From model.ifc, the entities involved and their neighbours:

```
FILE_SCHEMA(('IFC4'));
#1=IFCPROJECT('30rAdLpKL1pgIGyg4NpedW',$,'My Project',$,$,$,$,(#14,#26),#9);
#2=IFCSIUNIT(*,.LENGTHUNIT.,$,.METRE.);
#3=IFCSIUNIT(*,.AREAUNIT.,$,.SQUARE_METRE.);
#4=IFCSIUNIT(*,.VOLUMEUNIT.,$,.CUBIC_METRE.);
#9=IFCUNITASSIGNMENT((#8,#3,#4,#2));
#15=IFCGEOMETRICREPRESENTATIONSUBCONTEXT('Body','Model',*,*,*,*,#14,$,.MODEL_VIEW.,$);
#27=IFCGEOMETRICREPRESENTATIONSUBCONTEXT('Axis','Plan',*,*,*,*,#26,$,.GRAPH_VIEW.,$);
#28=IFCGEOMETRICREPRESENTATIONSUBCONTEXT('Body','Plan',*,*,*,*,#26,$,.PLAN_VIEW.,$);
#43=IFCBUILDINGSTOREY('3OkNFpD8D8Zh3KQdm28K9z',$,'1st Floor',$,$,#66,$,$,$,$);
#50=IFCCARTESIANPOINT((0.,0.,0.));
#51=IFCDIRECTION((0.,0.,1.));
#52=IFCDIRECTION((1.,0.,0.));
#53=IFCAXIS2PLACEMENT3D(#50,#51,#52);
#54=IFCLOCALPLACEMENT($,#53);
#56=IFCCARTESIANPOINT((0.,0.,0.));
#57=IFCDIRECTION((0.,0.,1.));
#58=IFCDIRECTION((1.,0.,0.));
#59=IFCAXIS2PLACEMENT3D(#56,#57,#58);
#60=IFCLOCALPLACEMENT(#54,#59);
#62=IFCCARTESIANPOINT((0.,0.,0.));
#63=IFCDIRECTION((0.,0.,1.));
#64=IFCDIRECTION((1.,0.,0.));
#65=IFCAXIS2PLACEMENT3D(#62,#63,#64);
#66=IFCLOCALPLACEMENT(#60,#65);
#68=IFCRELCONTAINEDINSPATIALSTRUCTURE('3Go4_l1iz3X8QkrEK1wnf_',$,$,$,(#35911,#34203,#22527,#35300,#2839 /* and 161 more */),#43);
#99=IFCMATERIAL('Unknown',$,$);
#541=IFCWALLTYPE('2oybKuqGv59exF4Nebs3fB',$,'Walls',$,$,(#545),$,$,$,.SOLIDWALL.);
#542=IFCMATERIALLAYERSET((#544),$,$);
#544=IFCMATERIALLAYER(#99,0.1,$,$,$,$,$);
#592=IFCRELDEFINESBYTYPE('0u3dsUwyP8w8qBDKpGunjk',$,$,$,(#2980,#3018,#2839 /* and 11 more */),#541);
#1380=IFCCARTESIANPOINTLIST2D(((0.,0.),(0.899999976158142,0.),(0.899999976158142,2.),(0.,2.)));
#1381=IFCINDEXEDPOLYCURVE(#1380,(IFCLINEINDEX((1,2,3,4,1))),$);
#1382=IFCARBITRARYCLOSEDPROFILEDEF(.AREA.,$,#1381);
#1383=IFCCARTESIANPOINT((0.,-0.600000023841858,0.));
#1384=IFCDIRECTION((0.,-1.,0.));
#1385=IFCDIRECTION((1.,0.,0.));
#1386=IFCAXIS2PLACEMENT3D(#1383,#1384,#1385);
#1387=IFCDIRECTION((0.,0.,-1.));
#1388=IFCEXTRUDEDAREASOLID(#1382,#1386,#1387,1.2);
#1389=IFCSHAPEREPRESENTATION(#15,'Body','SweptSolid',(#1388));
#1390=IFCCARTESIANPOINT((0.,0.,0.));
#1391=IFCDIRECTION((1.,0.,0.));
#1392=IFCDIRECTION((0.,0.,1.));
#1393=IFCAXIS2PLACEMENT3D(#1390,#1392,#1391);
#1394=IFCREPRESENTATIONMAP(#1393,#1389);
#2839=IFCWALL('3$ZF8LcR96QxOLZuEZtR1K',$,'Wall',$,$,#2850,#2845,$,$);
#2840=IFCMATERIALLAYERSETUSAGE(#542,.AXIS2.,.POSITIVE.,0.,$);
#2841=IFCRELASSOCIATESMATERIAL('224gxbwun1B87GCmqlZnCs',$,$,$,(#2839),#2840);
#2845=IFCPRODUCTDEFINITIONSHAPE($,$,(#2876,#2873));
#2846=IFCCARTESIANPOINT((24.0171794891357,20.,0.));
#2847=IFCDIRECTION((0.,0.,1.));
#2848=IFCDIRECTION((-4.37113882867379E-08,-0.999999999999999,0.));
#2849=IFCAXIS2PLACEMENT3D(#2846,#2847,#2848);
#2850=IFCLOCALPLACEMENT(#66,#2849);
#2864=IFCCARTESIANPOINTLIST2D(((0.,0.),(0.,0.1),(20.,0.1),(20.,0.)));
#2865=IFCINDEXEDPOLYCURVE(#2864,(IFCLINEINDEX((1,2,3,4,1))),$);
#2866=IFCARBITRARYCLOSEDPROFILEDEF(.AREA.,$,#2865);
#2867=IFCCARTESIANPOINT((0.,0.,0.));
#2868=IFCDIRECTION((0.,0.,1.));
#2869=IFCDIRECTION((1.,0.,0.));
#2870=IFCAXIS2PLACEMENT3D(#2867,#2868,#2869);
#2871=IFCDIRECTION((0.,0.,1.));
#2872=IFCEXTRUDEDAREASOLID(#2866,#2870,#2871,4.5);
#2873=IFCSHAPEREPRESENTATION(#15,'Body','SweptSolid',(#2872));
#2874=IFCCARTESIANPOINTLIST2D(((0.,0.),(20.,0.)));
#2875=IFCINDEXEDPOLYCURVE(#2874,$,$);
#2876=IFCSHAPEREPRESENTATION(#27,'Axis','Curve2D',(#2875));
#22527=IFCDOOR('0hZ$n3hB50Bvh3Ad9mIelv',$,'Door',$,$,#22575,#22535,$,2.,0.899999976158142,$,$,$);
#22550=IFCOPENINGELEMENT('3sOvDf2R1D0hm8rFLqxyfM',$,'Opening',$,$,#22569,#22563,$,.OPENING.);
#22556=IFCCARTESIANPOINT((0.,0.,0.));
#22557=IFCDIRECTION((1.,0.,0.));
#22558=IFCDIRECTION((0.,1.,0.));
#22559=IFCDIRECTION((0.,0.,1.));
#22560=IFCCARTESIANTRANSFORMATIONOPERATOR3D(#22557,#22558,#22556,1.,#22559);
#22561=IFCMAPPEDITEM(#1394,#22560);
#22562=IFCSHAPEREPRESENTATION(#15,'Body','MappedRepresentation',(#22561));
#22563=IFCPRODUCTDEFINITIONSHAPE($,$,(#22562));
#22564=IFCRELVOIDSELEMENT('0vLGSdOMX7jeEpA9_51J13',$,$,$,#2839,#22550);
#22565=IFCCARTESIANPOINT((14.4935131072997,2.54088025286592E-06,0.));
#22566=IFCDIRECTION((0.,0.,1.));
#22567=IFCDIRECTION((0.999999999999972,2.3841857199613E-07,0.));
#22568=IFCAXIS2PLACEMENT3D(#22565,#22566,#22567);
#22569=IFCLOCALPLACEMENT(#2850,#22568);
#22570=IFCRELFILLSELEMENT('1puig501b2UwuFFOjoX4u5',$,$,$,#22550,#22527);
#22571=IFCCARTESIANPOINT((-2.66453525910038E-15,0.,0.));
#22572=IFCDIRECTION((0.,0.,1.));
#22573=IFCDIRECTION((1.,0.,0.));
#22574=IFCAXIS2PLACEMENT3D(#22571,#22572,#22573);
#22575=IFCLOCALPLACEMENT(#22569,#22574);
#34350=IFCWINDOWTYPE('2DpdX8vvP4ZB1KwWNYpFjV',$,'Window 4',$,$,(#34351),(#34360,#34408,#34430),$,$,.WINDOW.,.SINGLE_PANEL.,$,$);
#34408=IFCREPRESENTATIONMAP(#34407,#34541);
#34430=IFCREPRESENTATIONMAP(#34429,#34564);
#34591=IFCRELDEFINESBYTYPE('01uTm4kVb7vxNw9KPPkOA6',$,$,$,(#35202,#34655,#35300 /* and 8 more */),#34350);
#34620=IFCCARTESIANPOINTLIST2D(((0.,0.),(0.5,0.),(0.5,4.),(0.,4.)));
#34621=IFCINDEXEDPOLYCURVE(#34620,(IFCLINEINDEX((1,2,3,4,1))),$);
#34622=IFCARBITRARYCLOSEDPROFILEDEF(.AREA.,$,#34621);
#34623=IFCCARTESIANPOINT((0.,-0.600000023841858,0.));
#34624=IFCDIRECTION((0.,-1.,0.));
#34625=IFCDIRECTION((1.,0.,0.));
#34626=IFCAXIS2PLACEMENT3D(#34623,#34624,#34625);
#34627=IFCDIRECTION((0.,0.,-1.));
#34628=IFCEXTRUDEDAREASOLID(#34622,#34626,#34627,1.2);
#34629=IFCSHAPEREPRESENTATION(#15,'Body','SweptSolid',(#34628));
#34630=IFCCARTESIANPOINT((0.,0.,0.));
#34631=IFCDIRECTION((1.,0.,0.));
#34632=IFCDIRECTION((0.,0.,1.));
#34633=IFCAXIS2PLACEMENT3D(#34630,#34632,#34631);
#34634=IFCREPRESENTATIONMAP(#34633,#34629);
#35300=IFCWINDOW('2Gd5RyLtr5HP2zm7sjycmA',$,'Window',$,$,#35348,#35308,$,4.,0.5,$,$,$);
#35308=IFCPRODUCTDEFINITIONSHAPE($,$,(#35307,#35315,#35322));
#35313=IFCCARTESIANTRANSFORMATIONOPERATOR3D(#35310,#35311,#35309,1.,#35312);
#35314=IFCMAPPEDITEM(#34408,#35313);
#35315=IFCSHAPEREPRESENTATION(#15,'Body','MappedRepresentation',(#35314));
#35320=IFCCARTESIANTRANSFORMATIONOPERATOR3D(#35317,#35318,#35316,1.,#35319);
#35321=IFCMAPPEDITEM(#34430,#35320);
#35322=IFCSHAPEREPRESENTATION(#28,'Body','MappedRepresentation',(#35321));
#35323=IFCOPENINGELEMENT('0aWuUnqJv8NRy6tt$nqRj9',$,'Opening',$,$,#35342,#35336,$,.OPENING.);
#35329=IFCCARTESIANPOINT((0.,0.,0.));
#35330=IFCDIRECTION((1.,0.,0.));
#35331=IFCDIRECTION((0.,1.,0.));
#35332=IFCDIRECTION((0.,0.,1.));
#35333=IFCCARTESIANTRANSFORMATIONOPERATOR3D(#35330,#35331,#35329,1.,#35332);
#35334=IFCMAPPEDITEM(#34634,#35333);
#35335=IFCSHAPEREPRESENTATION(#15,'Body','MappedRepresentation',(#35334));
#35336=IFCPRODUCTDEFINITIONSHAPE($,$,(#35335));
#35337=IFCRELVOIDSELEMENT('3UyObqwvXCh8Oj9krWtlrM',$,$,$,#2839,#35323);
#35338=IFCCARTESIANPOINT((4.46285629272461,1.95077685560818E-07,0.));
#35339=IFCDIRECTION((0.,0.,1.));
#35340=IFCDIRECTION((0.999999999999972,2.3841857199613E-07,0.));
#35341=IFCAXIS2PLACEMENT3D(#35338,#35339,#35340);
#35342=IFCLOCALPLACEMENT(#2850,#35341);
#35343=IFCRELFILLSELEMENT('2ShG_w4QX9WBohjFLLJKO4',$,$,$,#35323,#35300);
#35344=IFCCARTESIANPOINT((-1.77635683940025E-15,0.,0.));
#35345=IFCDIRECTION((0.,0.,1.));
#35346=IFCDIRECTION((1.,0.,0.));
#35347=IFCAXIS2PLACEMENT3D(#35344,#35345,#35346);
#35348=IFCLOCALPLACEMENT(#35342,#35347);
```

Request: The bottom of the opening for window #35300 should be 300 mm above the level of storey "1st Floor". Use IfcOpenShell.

```python
import numpy as np
import ifcopenshell
import ifcopenshell.api.geometry
import ifcopenshell.geom
import ifcopenshell.util.element
import ifcopenshell.util.placement
import ifcopenshell.util.shape
import ifcopenshell.util.unit

model = ifcopenshell.open("model.ifc")
unit_scale = ifcopenshell.util.unit.calculate_unit_scale(model)

window = model.by_guid("2Gd5RyLtr5HP2zm7sjycmA")
opening = window.FillsVoids[0].RelatingOpeningElement
storey = ifcopenshell.util.element.get_container(window, ifc_class="IfcBuildingStorey")
level = ifcopenshell.util.placement.get_local_placement(storey.ObjectPlacement)[2, 3]

# The opening's origin need not be at the sill, so measure its lowest point.
shape = ifcopenshell.geom.create_shape(ifcopenshell.geom.settings(), opening)
bottom = ifcopenshell.util.shape.get_shape_bottom_elevation(shape, shape.geometry) / unit_scale
dz = level + 0.3 / unit_scale - bottom

shift = np.array([0.0, 0.0, dz])
# The window is placed relative to its opening, so it follows when the opening moves.
matrix = ifcopenshell.util.placement.get_local_placement(opening.ObjectPlacement)
matrix[:3, 3] += shift
ifcopenshell.api.geometry.edit_object_placement(
    model, product=opening, matrix=matrix, is_si=False, should_transform_children=True
)

print(f"moved by {dz * unit_scale:+.3f} m")

model.write("model-out.ifc")
```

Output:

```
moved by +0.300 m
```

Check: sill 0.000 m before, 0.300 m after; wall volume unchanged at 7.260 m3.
